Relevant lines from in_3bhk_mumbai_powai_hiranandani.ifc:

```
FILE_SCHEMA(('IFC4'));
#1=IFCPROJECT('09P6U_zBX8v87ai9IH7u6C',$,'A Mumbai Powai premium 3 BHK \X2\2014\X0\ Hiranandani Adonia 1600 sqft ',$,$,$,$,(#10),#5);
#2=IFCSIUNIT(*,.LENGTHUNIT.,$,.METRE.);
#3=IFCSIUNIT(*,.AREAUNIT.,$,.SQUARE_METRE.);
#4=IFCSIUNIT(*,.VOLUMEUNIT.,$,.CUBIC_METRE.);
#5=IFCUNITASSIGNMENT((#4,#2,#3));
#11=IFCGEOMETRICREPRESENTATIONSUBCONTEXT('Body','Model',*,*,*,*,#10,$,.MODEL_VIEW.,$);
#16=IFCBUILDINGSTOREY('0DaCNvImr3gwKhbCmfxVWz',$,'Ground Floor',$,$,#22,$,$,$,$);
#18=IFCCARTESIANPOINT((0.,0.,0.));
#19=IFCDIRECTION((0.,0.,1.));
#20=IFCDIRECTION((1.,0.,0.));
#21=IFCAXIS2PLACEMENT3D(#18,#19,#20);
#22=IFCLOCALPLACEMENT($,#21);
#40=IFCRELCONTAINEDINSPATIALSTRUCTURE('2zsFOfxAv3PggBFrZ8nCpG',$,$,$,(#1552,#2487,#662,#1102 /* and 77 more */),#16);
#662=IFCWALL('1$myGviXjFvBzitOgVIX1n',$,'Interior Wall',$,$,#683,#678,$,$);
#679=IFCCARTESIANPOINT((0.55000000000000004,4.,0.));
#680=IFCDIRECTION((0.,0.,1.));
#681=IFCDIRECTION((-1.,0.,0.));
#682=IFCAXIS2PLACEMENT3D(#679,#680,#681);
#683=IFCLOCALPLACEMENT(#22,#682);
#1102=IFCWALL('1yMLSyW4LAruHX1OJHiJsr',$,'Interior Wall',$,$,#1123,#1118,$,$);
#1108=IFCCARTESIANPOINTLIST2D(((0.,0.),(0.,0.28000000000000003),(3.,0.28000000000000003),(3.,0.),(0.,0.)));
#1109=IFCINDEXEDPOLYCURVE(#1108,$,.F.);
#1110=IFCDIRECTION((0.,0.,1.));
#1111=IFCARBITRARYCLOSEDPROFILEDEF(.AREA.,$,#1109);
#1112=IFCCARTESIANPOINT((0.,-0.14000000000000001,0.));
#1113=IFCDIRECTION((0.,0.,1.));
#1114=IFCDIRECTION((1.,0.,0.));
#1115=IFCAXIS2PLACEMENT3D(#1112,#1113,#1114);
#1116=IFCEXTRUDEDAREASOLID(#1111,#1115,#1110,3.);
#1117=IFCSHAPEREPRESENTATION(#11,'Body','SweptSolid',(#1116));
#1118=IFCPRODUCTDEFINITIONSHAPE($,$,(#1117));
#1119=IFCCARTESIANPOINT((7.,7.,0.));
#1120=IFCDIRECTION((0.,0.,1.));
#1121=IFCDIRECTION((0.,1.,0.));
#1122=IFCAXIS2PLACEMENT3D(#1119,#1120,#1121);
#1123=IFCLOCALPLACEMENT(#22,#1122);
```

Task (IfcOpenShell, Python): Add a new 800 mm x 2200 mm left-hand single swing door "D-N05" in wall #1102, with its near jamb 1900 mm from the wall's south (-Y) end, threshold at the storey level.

```python
import numpy as np
import ifcopenshell
import ifcopenshell.api.feature
import ifcopenshell.api.geometry
import ifcopenshell.api.root
import ifcopenshell.api.spatial
import ifcopenshell.geom
import ifcopenshell.util.element
import ifcopenshell.util.placement
import ifcopenshell.util.representation
import ifcopenshell.util.shape
import ifcopenshell.util.unit

model = ifcopenshell.open("in_3bhk_mumbai_powai_hiranandani.ifc")
unit_scale = ifcopenshell.util.unit.calculate_unit_scale(model)
settings = ifcopenshell.geom.settings()


def volume(element):
    """Net volume in cubic metres, openings subtracted."""
    shape = ifcopenshell.geom.create_shape(settings, element)
    return ifcopenshell.util.shape.get_volume(shape.geometry)


wall = model.by_guid("1yMLSyW4LAruHX1OJHiJsr")
storey = ifcopenshell.util.element.get_container(wall, ifc_class="IfcBuildingStorey")
context = ifcopenshell.util.representation.get_context(model, "Model", "Body", "MODEL_VIEW")
before = volume(wall)

width, height, from_end, sill = 0.8, 2.2, 1.9, 0.0  # metres

# The wall runs along its own X axis, and the end named is its -X end.
wall_shape = ifcopenshell.geom.create_shape(settings, wall)
x, y, z = ifcopenshell.util.shape.get_vertices(wall_shape.geometry).T
start = x.min() + from_end
face, thickness = float(y.min()), float(y.max() - y.min())
wall_matrix = ifcopenshell.util.placement.get_local_placement(wall.ObjectPlacement)
level = ifcopenshell.util.placement.get_local_placement(storey.ObjectPlacement)[2, 3]


def in_wall(x, y):
    """Placement at x, y metres in the wall's axes, at sill height."""
    matrix = wall_matrix.copy()
    matrix[:, 3] = wall_matrix @ np.array([x / unit_scale, y / unit_scale, 0.0, 1.0])
    matrix[2, 3] = level + sill / unit_scale
    return matrix


# Opening: a box that overshoots both wall faces by 50 mm.
opening = ifcopenshell.api.root.create_entity(model, ifc_class="IfcOpeningElement", predefined_type="OPENING")
box = ifcopenshell.api.geometry.add_wall_representation(
    model, context=context, length=width, height=height, thickness=thickness + 0.1
)
ifcopenshell.api.geometry.assign_representation(model, product=opening, representation=box)
ifcopenshell.api.geometry.edit_object_placement(model, product=opening, matrix=in_wall(start, face - 0.05), is_si=False)
ifcopenshell.api.feature.add_feature(model, feature=opening, element=wall)

door = ifcopenshell.api.root.create_entity(model, ifc_class="IfcDoor", name="D-N05", predefined_type="DOOR")
door.OverallWidth, door.OverallHeight = width / unit_scale, height / unit_scale
door.OperationType = "SINGLE_SWING_LEFT"
body = ifcopenshell.api.geometry.add_door_representation(
    model,
    context=context,
    overall_width=door.OverallWidth,
    overall_height=door.OverallHeight,
    operation_type="SINGLE_SWING_LEFT",
    lining_properties={"LiningDepth": thickness / unit_scale, "ThresholdDepth": thickness / unit_scale},
)
ifcopenshell.api.geometry.assign_representation(model, product=door, representation=body)
ifcopenshell.api.spatial.assign_container(model, products=[door], relating_structure=storey)
ifcopenshell.api.feature.add_filling(model, opening=opening, element=door)

# The lining spans the wall, so the door starts at the wall face.
ifcopenshell.api.geometry.edit_object_placement(model, product=door, matrix=in_wall(start, face), is_si=False)

after = volume(wall)

print(f"wall volume {before:.3f} -> {after:.3f} m3")

model.write("in_3bhk_mumbai_powai_hiranandani_updated.ifc")
```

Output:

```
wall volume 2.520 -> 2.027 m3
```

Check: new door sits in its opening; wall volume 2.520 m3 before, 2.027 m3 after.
